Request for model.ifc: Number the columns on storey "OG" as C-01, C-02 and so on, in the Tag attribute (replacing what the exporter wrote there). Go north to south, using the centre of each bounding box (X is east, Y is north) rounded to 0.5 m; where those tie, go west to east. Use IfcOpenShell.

First a look at what the model holds.

```python
import ifcopenshell
import ifcopenshell.util.element
import ifcopenshell.util.placement

model = ifcopenshell.open("model.ifc")
print(model.schema)
storey = next(s for s in model.by_type("IfcBuildingStorey") if s.Name == "OG")
columns = [e for e in ifcopenshell.util.element.get_decomposition(storey) if e.is_a("IfcColumn")]
for e in sorted(columns, key=lambda e: e.id()):
    origin = ifcopenshell.util.placement.get_local_placement(e.ObjectPlacement)[:3, 3]
    print(e.id(), e.Tag, e.Name, origin.round(2) + 0.0, sep=" | ")
```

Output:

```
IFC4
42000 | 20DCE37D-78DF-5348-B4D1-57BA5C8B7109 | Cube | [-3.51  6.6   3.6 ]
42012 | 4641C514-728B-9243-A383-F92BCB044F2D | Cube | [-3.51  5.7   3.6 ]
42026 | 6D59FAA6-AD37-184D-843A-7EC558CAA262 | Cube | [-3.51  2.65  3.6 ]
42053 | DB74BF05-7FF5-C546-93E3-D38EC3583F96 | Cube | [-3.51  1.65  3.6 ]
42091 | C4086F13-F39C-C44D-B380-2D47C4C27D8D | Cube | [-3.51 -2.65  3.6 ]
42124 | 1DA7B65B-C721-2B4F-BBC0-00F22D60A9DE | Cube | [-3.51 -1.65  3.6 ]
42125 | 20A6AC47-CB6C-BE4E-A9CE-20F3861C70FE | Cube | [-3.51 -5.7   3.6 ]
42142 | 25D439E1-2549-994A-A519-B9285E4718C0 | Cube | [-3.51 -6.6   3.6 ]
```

```python
import ifcopenshell
import ifcopenshell.geom
import ifcopenshell.util.element
import ifcopenshell.util.shape

model = ifcopenshell.open("model.ifc")
settings = ifcopenshell.geom.settings()
settings.set("use-world-coords", True)


def centre(element):
    shape = ifcopenshell.geom.create_shape(settings, element)
    return ifcopenshell.util.shape.get_bbox_centroid(shape.geometry)


storey = next(s for s in model.by_type("IfcBuildingStorey") if s.Name == "OG")
columns = [e for e in ifcopenshell.util.element.get_decomposition(storey) if e.is_a("IfcColumn")]

# Insertion points can sit at a corner or the storey origin, so sort by the geometry (in metres).
centres = {e: centre(e) for e in columns}
columns.sort(key=lambda e: (-round(centres[e][1] / 0.5), centres[e][0]))

for i, e in enumerate(columns, start=1):
    number = f"C-{i:02d}"
    e.Tag = number
    print(e.id(), number)

model.write("model_edited.ifc")
```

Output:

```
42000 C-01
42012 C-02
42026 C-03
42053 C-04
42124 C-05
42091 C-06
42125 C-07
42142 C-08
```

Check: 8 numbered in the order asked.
